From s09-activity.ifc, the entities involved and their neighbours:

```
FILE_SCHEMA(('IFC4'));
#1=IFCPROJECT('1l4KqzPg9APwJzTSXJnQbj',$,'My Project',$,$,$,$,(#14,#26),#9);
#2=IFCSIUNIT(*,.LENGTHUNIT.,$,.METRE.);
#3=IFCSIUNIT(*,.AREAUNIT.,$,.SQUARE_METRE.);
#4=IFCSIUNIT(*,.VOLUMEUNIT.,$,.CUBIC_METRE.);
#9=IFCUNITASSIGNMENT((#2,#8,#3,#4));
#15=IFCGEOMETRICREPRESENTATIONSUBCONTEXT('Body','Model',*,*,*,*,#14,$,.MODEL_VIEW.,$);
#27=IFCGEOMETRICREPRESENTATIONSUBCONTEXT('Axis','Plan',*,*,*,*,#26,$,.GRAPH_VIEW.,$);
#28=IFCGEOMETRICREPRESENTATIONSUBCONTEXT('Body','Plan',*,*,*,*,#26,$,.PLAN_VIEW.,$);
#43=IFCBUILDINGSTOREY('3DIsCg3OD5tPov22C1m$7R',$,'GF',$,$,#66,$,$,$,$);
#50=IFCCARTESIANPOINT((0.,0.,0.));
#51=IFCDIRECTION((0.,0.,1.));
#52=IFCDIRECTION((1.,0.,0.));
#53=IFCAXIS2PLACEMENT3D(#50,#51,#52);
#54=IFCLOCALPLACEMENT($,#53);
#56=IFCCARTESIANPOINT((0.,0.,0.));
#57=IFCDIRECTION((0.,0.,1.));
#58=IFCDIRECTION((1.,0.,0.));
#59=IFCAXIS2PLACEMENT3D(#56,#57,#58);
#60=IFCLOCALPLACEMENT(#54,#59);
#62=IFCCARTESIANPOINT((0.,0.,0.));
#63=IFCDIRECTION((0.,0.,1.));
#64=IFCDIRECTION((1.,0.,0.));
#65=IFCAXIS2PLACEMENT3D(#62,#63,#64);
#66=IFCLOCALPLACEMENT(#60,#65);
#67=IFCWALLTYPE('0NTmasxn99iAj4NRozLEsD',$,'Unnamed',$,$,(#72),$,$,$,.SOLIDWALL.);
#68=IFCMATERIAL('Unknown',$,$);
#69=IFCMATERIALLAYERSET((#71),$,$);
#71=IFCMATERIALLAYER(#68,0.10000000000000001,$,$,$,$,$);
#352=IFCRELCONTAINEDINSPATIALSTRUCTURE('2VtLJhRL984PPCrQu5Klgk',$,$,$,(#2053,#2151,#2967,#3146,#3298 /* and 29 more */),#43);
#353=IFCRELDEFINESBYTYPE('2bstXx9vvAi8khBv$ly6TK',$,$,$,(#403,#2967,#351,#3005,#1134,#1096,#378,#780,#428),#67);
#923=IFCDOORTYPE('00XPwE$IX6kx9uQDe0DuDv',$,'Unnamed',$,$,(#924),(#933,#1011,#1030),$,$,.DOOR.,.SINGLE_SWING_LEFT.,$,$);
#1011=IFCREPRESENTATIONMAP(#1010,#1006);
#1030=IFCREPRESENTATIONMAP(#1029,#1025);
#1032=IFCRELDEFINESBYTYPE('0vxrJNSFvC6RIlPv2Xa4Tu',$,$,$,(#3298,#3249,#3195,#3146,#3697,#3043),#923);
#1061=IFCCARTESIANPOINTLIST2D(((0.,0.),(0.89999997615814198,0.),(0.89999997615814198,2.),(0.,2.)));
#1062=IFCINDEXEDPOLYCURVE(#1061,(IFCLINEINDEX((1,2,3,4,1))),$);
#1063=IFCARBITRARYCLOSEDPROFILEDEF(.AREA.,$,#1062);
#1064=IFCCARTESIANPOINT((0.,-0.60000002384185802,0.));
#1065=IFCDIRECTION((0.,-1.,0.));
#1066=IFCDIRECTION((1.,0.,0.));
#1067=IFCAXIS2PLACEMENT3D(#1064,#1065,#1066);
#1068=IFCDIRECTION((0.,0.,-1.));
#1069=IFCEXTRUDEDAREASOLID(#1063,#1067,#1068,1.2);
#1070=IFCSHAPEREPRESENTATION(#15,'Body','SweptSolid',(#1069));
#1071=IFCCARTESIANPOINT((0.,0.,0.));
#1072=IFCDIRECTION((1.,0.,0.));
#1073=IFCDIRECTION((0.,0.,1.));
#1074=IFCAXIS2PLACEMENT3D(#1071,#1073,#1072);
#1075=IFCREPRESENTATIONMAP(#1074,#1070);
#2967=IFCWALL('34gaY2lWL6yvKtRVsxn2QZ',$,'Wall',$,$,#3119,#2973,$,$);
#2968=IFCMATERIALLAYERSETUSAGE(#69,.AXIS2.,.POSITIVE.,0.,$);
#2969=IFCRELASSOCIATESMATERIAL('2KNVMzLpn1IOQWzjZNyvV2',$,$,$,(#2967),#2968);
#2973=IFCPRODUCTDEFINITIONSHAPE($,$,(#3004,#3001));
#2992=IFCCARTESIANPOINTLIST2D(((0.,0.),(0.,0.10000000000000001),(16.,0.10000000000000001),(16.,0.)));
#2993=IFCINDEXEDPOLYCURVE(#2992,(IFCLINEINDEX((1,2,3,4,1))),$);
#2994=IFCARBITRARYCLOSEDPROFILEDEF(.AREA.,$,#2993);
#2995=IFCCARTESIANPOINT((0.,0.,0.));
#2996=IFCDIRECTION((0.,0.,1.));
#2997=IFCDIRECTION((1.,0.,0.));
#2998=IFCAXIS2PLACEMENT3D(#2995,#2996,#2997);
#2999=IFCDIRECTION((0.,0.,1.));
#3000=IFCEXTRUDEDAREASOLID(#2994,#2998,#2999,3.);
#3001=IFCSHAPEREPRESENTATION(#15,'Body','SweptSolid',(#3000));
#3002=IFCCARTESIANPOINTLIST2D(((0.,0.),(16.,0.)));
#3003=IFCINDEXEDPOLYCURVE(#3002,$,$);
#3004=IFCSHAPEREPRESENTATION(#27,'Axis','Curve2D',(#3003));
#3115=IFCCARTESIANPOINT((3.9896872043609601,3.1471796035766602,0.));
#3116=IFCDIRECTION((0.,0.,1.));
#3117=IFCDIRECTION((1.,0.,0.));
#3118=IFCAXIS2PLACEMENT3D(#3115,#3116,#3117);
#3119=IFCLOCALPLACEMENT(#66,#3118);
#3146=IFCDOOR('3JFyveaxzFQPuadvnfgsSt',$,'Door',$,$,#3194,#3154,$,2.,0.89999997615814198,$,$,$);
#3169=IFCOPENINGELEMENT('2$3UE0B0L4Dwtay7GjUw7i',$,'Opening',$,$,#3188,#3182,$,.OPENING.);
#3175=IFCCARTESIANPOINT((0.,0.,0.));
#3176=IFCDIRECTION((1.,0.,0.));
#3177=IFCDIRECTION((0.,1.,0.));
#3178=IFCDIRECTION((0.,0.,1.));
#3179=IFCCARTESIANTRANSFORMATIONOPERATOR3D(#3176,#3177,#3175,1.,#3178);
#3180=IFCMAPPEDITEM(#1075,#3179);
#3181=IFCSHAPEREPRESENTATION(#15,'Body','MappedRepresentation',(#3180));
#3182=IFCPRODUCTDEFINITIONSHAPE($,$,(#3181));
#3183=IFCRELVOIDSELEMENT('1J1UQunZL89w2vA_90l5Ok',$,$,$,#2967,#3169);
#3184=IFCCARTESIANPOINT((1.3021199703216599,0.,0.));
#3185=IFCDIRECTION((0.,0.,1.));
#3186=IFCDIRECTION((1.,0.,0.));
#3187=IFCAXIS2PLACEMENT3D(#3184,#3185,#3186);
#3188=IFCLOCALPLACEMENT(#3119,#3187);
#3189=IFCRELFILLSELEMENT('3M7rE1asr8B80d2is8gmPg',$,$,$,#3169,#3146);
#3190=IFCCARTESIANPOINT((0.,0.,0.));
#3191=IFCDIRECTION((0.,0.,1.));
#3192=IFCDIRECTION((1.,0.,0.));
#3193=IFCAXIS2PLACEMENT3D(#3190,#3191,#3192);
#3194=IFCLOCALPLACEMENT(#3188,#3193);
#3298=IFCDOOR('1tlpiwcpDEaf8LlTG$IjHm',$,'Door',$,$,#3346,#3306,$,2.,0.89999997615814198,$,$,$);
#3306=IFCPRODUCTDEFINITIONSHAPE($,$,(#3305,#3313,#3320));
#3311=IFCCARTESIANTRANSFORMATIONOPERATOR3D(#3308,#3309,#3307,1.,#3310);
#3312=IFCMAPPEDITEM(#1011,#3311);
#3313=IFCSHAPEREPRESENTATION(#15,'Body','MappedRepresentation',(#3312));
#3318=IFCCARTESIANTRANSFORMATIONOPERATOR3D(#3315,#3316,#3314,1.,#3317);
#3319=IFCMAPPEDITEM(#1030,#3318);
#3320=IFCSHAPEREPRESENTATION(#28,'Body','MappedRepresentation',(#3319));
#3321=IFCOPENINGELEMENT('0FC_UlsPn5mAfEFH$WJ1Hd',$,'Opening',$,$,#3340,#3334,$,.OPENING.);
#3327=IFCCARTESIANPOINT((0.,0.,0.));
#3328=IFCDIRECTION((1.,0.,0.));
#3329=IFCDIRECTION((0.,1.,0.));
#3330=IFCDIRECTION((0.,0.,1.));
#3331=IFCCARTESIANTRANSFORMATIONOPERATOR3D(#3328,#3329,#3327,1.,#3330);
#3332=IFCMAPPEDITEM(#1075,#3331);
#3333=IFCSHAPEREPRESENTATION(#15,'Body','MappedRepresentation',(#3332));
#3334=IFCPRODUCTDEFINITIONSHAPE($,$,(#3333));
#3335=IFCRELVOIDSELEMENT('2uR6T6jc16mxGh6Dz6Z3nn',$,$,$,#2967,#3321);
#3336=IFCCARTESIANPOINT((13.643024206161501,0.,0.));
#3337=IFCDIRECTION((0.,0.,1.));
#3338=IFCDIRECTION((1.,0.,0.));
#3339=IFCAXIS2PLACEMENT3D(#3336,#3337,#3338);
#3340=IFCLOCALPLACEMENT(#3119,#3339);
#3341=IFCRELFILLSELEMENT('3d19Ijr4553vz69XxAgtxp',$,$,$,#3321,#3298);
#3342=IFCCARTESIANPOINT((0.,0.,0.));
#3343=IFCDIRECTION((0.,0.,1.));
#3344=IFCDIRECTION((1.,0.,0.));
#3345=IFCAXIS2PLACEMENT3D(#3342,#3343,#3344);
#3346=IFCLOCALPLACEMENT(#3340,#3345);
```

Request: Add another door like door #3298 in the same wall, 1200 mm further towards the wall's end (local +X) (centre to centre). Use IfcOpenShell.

```python
import ifcopenshell
import ifcopenshell.api.feature
import ifcopenshell.api.geometry
import ifcopenshell.api.root
import ifcopenshell.geom
import ifcopenshell.util.element
import ifcopenshell.util.placement
import ifcopenshell.util.shape

model = ifcopenshell.open("s09-activity.ifc")
settings = ifcopenshell.geom.settings()


def volume(element):
    """Net volume in cubic metres, openings subtracted."""
    shape = ifcopenshell.geom.create_shape(settings, element)
    return ifcopenshell.util.shape.get_volume(shape.geometry)


door = model.by_guid("1tlpiwcpDEaf8LlTG$IjHm")
opening = door.FillsVoids[0].RelatingOpeningElement
wall = opening.VoidsElements[0].RelatingBuildingElement
before = volume(wall)
shift = ifcopenshell.util.placement.get_local_placement(wall.ObjectPlacement)[:3, 0] * 1.2

# copy_class copies the void relationship, type, container and properties, but no geometry.
new_opening = ifcopenshell.api.root.copy_class(model, product=opening)
new_opening.Representation = ifcopenshell.util.element.copy_deep(
    model, opening.Representation, exclude=["IfcGeometricRepresentationContext", "IfcRepresentationMap"]
)
new_door = ifcopenshell.api.root.copy_class(model, product=door)
new_door.Representation = ifcopenshell.util.element.copy_deep(
    model, door.Representation, exclude=["IfcGeometricRepresentationContext", "IfcRepresentationMap"]
)
ifcopenshell.api.feature.add_filling(model, opening=new_opening, element=new_door)

for old, new in ((opening, new_opening), (door, new_door)):
    matrix = ifcopenshell.util.placement.get_local_placement(old.ObjectPlacement)
    matrix[:3, 3] += shift
    ifcopenshell.api.geometry.edit_object_placement(model, product=new, matrix=matrix, is_si=False)

after = volume(wall)

print(f"wall volume {before:.3f} -> {after:.3f} m3")

model.write("s09-activity_updated.ifc")
```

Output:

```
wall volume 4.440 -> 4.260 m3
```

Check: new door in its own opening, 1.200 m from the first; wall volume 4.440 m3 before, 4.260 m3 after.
